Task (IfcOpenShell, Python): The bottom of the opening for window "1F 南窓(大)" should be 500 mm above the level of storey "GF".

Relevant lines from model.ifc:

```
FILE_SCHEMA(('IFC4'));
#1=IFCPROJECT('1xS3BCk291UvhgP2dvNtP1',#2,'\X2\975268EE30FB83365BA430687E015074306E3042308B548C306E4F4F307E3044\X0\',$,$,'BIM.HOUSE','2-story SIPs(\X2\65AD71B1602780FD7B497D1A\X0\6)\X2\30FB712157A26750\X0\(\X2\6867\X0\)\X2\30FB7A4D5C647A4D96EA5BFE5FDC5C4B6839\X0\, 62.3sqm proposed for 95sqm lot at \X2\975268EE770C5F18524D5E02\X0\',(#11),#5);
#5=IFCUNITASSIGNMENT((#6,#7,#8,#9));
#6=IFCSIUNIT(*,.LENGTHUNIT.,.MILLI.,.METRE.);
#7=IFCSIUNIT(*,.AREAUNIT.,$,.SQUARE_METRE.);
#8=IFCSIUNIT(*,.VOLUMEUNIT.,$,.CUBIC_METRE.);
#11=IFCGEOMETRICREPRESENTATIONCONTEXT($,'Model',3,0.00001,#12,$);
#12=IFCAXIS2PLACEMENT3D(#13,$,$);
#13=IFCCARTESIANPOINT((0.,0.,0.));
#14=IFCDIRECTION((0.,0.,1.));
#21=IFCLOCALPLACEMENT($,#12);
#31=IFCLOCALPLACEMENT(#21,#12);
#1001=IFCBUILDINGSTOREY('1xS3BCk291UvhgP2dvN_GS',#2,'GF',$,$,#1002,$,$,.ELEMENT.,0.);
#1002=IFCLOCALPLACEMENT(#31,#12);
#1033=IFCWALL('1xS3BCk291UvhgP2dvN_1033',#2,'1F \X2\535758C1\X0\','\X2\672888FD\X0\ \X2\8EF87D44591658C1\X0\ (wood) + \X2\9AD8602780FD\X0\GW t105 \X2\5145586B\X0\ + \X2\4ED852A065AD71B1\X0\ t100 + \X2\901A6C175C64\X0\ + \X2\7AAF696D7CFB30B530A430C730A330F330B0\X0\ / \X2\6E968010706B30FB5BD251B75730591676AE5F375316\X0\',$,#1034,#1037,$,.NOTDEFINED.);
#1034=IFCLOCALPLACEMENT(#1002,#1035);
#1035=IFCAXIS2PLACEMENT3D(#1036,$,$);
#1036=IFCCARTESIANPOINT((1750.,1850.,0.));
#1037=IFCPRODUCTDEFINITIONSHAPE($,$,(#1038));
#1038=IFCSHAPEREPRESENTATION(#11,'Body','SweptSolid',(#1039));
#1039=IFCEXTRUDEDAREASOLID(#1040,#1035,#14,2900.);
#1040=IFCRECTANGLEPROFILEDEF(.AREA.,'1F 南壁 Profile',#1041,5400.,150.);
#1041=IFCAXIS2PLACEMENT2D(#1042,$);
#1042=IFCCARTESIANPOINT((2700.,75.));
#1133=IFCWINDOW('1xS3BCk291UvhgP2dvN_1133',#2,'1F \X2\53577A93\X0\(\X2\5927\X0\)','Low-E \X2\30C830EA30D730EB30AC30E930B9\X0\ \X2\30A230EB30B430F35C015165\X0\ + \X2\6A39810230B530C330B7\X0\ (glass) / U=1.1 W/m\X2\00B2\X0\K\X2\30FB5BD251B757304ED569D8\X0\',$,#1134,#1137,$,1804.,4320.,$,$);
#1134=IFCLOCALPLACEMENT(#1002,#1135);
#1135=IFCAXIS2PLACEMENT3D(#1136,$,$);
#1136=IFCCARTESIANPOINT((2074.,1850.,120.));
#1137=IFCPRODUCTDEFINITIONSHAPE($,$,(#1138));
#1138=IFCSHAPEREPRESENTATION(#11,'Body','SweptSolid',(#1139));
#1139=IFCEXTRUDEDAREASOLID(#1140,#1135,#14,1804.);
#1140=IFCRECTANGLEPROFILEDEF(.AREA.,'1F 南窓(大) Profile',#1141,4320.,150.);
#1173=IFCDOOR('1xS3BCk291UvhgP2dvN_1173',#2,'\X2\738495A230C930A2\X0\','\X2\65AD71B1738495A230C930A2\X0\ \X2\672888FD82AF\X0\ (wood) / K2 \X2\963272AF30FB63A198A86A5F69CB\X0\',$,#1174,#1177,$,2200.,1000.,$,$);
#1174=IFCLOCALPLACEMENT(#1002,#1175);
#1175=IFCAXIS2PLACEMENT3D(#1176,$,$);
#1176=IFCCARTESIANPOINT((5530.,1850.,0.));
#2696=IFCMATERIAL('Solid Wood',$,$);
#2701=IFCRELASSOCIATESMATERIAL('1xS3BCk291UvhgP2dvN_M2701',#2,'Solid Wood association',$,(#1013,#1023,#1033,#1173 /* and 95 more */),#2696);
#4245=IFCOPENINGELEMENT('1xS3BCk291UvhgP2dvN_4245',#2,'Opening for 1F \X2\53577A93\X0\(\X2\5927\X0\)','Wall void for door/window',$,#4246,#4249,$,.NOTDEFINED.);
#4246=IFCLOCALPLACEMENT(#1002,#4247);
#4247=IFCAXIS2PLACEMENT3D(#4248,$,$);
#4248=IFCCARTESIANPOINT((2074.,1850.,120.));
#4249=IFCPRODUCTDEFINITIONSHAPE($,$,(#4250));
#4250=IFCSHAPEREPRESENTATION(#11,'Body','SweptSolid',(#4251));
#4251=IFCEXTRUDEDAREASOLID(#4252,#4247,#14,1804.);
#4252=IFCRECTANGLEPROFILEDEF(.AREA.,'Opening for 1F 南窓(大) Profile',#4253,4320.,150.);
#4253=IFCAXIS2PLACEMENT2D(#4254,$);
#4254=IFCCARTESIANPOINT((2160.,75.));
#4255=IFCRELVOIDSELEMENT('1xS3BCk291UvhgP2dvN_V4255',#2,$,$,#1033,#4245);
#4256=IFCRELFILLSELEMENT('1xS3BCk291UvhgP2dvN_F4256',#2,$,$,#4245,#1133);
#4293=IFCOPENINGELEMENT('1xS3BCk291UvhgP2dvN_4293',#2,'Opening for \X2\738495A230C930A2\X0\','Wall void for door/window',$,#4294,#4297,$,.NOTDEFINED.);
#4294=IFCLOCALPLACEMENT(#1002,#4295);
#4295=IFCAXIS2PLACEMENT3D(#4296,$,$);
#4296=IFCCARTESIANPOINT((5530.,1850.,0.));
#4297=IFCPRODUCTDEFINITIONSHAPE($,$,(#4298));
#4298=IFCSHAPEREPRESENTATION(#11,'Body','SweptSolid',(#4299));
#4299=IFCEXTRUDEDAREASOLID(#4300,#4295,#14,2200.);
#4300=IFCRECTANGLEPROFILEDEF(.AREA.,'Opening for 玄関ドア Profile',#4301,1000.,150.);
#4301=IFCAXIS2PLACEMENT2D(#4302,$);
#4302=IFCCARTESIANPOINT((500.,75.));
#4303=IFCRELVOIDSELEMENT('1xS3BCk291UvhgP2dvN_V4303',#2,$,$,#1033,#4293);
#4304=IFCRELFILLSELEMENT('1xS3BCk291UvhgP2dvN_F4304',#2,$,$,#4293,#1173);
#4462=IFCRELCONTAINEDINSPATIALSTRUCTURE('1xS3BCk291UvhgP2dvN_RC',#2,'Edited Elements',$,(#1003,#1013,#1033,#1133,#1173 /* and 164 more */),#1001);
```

```python
import numpy as np
import ifcopenshell
import ifcopenshell.api.geometry
import ifcopenshell.geom
import ifcopenshell.util.element
import ifcopenshell.util.placement
import ifcopenshell.util.shape
import ifcopenshell.util.unit

model = ifcopenshell.open("model.ifc")
unit_scale = ifcopenshell.util.unit.calculate_unit_scale(model)

window = model.by_guid("1xS3BCk291UvhgP2dvN_1133")
opening = window.FillsVoids[0].RelatingOpeningElement
storey = ifcopenshell.util.element.get_container(window, ifc_class="IfcBuildingStorey")
level = ifcopenshell.util.placement.get_local_placement(storey.ObjectPlacement)[2, 3]

# The opening's origin need not be at the sill, so measure its lowest point.
shape = ifcopenshell.geom.create_shape(ifcopenshell.geom.settings(), opening)
bottom = ifcopenshell.util.shape.get_shape_bottom_elevation(shape, shape.geometry) / unit_scale
dz = level + 500.0 - bottom

shift = np.array([0.0, 0.0, dz])
# The window is not placed relative to its opening, so move both.
for product in (opening, window):
    matrix = ifcopenshell.util.placement.get_local_placement(product.ObjectPlacement)
    matrix[:3, 3] += shift
    ifcopenshell.api.geometry.edit_object_placement(model, product=product, matrix=matrix, is_si=False)

print(f"moved by {dz * unit_scale:+.3f} m")

model.write("model_edited.ifc")
```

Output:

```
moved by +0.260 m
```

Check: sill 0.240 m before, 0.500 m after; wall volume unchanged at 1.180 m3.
